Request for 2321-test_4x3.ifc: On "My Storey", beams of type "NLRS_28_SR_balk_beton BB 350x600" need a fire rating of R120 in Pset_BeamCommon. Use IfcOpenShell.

First a look at what the model holds.

```python
import ifcopenshell
import ifcopenshell.util.element

model = ifcopenshell.open("2321-test_4x3.ifc")
print(model.schema)
storey = next(s for s in model.by_type("IfcBuildingStorey") if s.Name == "My Storey")
beams = [e for e in ifcopenshell.util.element.get_decomposition(storey) if e.is_a("IfcBeam")]
seen = {}
for e in beams:
    element_type = ifcopenshell.util.element.get_type(e)
    key = (element_type.Name if element_type != e and element_type else None, ifcopenshell.util.element.get_pset(e, "Pset_BeamCommon", "FireRating"))
    seen[key] = seen.get(key, 0) + 1
for (name, value), count in sorted(seen.items(), key=str):
    print(count, "x", name, "|", value)
```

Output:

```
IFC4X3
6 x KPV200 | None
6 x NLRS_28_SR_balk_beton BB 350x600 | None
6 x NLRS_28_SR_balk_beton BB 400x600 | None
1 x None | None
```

```python
import ifcopenshell
import ifcopenshell.api.pset
import ifcopenshell.util.element

model = ifcopenshell.open("2321-test_4x3.ifc")

storey = next(s for s in model.by_type("IfcBuildingStorey") if s.Name == "My Storey")
beams = [e for e in ifcopenshell.util.element.get_decomposition(storey) if e.is_a("IfcBeam")]

count = 0
for e in beams:
    element_type = ifcopenshell.util.element.get_type(e)
    if element_type in (None, e) or element_type.Name != "NLRS_28_SR_balk_beton BB 350x600":
        continue
    # add_pset returns the element's existing set when there is one.
    pset = ifcopenshell.api.pset.add_pset(model, product=e, name="Pset_BeamCommon")
    ifcopenshell.api.pset.edit_pset(model, pset=pset, properties={"FireRating": "R120"})
    count += 1

print(count, "beams updated")

model.write("2321-test_4x3_updated.ifc")
```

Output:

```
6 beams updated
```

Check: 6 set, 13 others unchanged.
